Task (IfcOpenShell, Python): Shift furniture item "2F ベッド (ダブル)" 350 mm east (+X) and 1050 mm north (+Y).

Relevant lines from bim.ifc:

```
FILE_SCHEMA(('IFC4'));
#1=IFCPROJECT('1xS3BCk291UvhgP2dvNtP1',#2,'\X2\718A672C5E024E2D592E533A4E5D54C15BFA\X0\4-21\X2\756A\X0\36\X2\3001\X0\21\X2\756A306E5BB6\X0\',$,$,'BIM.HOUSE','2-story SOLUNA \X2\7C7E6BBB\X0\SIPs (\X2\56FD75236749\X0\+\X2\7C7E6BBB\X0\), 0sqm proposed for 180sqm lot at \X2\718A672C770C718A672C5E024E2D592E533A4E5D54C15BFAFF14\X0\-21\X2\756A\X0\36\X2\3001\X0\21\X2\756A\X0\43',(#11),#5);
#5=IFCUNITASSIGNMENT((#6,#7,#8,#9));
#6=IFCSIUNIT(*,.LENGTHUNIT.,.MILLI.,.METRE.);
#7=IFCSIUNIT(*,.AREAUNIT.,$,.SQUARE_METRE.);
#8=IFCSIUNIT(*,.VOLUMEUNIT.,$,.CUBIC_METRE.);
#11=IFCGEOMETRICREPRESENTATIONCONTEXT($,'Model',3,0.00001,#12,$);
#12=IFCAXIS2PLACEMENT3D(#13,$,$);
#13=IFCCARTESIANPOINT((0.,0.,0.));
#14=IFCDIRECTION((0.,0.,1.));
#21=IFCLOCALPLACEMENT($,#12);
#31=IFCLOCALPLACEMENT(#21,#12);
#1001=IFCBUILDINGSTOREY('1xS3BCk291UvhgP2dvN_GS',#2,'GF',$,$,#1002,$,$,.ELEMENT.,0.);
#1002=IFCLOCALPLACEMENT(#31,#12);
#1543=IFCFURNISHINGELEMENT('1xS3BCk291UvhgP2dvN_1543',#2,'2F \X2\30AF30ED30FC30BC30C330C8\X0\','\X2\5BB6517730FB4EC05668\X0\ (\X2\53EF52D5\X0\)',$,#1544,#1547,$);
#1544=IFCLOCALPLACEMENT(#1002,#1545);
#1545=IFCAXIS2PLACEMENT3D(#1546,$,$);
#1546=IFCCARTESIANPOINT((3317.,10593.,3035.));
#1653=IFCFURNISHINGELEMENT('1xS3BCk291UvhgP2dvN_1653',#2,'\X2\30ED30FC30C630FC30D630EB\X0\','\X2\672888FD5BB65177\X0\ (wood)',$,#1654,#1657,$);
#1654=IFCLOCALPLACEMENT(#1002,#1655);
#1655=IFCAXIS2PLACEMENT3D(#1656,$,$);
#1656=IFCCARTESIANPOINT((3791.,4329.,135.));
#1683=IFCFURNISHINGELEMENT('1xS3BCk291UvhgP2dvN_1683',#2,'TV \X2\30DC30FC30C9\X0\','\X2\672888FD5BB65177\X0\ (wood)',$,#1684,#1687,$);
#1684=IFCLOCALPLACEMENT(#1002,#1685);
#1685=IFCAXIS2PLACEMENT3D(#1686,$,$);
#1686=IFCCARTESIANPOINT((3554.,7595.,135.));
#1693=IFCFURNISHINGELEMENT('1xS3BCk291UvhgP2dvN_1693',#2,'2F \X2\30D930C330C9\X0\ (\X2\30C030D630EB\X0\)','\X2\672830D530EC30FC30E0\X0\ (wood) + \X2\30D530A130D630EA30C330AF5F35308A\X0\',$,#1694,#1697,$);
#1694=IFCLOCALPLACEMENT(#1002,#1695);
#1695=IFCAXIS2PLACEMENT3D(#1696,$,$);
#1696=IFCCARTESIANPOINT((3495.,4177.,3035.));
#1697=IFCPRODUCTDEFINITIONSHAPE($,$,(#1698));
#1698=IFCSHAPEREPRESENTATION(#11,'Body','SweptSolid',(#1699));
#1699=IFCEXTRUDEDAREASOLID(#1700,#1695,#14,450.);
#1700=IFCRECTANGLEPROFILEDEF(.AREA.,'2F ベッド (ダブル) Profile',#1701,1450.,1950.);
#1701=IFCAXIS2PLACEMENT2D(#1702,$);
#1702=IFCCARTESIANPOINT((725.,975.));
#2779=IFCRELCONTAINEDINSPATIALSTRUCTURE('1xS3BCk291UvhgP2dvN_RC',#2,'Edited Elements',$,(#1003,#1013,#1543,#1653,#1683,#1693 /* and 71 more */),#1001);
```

```python
import ifcopenshell
import ifcopenshell.api.geometry
import ifcopenshell.util.placement
import ifcopenshell.util.unit

model = ifcopenshell.open("bim.ifc")
unit_scale = ifcopenshell.util.unit.calculate_unit_scale(model)

item = model.by_guid("1xS3BCk291UvhgP2dvN_1693")
matrix = ifcopenshell.util.placement.get_local_placement(item.ObjectPlacement)
matrix[0, 3] += 0.35 / unit_scale
matrix[1, 3] += 1.05 / unit_scale
ifcopenshell.api.geometry.edit_object_placement(model, product=item, matrix=matrix, is_si=False)

print(ifcopenshell.util.placement.get_local_placement(item.ObjectPlacement).round(3) + 0.0)

model.write("bim_edited.ifc")
```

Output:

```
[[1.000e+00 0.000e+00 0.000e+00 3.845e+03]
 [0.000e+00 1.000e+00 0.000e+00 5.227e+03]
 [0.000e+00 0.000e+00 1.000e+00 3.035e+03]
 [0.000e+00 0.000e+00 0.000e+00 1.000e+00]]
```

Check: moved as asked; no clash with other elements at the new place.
